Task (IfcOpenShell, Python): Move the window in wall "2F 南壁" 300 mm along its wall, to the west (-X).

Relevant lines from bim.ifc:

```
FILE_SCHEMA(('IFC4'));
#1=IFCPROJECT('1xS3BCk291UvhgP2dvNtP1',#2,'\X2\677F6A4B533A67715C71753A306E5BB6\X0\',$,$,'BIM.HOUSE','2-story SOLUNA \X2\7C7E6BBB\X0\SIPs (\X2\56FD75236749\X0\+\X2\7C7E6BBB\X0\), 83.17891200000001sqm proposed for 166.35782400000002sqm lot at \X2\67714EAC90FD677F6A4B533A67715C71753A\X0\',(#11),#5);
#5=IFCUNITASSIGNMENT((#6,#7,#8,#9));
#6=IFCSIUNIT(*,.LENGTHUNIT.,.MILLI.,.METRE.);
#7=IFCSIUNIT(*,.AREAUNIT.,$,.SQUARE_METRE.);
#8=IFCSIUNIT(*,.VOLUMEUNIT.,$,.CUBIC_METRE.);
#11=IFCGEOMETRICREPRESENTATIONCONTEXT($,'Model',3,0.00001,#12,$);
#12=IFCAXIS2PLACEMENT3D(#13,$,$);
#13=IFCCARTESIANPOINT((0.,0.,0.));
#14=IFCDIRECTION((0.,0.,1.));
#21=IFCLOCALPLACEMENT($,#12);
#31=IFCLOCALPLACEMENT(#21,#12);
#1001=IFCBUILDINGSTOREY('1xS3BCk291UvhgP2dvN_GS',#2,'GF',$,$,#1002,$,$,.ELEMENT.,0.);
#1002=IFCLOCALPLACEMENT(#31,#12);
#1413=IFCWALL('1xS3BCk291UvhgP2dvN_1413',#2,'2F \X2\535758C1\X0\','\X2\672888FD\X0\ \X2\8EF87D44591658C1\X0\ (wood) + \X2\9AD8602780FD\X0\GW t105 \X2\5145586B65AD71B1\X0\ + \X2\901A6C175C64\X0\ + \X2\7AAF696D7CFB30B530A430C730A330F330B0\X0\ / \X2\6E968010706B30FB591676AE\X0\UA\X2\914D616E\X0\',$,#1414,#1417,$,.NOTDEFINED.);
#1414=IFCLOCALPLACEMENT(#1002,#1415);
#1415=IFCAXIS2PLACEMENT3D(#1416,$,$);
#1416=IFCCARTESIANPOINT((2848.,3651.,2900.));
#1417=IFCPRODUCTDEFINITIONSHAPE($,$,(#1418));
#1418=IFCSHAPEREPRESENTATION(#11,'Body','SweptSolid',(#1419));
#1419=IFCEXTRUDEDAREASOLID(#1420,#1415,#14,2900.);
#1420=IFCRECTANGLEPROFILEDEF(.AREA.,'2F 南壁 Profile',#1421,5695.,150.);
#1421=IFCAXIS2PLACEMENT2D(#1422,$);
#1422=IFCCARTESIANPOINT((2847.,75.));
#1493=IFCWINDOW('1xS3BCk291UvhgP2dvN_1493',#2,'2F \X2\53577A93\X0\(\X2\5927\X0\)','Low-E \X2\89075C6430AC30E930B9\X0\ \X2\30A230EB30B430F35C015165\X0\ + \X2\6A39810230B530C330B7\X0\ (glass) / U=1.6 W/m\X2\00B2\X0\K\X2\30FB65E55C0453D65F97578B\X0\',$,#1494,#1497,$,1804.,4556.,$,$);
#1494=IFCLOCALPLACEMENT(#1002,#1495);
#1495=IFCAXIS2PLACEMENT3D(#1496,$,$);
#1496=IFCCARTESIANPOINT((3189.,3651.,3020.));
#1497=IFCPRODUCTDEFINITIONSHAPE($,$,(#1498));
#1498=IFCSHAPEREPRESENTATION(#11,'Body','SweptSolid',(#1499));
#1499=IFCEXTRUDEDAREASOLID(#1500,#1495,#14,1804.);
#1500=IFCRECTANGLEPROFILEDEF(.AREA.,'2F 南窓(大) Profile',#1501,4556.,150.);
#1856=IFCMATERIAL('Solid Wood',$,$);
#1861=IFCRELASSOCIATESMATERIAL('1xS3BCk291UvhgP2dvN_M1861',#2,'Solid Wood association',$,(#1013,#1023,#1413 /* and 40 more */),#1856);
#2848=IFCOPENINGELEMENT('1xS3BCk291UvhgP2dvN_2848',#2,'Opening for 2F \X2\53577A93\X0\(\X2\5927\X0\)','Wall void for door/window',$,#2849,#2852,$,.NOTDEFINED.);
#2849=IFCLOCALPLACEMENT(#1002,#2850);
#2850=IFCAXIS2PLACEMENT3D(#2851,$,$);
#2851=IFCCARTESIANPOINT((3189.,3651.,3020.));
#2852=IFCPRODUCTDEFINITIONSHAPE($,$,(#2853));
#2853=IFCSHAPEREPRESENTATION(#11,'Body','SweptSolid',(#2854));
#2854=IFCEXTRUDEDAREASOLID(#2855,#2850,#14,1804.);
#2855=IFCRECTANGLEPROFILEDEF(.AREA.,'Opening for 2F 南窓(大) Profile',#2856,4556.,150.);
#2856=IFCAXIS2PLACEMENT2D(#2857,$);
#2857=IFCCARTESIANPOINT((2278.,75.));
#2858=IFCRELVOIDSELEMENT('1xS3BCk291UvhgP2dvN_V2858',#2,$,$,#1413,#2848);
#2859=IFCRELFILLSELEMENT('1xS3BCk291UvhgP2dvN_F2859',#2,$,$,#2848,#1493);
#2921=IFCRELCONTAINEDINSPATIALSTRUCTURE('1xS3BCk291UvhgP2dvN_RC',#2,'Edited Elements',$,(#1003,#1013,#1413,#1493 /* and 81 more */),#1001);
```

```python
import ifcopenshell
import ifcopenshell.api.geometry
import ifcopenshell.util.placement

model = ifcopenshell.open("bim.ifc")

window = model.by_guid("1xS3BCk291UvhgP2dvN_1493")
opening = window.FillsVoids[0].RelatingOpeningElement
wall = opening.VoidsElements[0].RelatingBuildingElement

wall_matrix = ifcopenshell.util.placement.get_local_placement(wall.ObjectPlacement)
shift = wall_matrix[:3, 0] * -300.0
before = ifcopenshell.util.placement.get_local_placement(window.ObjectPlacement)[:3, 3].copy()

# The window is not placed relative to its opening, so move both.
for product in (opening, window):
    matrix = ifcopenshell.util.placement.get_local_placement(product.ObjectPlacement)
    matrix[:3, 3] += shift
    ifcopenshell.api.geometry.edit_object_placement(model, product=product, matrix=matrix, is_si=False)

after = ifcopenshell.util.placement.get_local_placement(window.ObjectPlacement)[:3, 3]
print("window moved by", (after - before).round(3) + 0.0)

model.write("bim_rev.ifc")
```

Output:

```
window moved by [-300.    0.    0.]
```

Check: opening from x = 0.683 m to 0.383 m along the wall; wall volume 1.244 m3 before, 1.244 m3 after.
